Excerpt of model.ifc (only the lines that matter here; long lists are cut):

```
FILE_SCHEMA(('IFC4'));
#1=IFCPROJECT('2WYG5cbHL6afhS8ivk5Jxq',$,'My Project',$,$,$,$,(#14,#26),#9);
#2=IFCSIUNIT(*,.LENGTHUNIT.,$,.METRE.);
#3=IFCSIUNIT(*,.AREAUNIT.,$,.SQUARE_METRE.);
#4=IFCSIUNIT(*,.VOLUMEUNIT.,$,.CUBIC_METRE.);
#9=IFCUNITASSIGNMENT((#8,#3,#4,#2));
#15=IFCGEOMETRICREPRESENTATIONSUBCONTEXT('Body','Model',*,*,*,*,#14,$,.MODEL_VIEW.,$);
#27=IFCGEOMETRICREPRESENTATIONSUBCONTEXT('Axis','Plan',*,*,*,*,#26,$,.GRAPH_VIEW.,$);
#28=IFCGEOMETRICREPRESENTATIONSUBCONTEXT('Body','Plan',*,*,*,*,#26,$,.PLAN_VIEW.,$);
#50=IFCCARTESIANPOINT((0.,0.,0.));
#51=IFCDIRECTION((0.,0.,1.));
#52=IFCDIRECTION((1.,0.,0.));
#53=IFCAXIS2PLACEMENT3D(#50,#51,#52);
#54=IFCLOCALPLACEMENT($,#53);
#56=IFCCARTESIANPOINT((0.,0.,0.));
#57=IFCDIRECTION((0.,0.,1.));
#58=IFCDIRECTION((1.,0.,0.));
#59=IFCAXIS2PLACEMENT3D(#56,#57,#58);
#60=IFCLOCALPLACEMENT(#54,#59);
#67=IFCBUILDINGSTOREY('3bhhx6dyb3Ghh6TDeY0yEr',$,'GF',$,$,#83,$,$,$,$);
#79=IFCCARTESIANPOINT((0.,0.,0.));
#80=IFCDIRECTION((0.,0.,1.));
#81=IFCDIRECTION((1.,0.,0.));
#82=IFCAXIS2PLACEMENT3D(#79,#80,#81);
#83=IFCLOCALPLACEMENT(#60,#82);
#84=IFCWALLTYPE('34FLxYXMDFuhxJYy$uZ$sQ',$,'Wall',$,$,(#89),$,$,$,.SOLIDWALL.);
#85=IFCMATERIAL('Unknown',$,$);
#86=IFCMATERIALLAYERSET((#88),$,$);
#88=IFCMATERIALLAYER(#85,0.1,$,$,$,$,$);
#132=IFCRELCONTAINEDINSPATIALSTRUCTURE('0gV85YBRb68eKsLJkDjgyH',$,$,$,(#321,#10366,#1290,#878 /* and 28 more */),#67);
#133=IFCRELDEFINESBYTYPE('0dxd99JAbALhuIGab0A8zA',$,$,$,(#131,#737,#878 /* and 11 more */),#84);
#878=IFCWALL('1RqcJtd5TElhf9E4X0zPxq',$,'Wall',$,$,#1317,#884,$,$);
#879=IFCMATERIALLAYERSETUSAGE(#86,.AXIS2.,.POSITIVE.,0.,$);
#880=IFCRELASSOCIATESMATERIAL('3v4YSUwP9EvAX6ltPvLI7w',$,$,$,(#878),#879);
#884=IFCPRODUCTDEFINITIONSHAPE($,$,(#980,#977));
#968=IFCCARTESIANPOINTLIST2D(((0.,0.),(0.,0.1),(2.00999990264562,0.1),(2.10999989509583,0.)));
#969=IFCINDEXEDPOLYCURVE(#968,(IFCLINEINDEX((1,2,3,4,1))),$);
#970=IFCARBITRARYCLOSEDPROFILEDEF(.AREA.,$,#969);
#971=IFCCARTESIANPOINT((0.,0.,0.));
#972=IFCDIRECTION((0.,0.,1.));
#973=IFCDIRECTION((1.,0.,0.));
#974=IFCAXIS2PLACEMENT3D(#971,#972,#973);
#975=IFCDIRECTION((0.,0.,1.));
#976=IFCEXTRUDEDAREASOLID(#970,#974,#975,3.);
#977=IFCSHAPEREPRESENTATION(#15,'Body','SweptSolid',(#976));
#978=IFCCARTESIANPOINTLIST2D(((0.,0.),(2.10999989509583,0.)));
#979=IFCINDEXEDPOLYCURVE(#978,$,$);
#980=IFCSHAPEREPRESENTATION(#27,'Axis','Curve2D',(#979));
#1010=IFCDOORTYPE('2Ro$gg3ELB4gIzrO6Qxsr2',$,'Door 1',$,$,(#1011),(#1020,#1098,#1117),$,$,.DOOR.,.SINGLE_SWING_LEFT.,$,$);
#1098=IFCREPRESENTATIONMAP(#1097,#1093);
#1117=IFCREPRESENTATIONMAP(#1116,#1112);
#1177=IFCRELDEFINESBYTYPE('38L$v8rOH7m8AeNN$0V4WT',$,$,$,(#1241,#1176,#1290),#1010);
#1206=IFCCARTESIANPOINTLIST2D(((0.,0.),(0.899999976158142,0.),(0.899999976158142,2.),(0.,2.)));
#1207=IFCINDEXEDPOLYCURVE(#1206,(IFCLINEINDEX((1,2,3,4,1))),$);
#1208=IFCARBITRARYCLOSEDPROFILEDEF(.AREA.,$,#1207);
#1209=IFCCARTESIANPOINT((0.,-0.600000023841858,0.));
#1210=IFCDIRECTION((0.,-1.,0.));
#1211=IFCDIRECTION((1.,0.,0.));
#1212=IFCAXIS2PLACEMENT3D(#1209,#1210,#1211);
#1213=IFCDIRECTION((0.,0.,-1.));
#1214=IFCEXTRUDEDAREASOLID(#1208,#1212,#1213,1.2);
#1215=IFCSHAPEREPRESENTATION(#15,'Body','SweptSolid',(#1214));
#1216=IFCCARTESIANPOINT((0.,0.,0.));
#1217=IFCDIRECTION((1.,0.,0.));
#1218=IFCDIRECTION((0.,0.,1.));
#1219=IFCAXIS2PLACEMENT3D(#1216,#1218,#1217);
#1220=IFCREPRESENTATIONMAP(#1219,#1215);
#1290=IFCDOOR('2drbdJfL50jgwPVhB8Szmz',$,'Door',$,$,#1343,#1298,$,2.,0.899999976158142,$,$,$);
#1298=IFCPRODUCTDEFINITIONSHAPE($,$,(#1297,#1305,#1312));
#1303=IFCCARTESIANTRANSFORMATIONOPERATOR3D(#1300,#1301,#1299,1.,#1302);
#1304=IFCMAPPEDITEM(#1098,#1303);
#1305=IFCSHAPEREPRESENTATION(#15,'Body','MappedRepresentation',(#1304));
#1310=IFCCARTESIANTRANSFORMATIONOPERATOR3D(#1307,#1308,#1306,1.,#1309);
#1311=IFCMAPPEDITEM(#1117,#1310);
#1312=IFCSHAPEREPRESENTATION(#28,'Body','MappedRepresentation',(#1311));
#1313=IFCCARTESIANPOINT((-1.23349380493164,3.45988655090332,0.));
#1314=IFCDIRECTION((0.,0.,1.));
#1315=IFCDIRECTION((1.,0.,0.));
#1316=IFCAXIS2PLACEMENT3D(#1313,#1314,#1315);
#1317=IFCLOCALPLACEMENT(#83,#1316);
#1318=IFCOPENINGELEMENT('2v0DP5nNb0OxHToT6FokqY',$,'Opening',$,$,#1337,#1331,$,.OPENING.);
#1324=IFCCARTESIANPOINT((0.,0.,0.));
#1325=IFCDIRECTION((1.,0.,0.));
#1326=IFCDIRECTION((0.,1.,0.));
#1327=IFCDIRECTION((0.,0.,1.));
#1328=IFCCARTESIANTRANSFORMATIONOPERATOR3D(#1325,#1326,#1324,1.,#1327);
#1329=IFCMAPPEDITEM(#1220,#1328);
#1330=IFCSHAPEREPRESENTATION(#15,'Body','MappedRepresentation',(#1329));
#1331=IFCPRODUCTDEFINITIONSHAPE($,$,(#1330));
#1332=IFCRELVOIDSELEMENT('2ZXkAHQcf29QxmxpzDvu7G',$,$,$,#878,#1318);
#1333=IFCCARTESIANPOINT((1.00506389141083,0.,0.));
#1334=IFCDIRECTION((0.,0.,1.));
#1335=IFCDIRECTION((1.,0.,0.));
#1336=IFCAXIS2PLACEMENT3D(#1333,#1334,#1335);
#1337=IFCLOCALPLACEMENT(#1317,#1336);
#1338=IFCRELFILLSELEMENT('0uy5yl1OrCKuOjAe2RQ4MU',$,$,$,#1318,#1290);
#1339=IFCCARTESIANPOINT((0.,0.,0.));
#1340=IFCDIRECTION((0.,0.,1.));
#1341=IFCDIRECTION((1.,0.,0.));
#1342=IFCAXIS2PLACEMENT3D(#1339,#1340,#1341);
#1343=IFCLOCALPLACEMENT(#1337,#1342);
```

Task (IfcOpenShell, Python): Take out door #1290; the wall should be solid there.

```python
import ifcopenshell
import ifcopenshell.api.feature
import ifcopenshell.api.root
import ifcopenshell.geom
import ifcopenshell.util.shape

model = ifcopenshell.open("model.ifc")
settings = ifcopenshell.geom.settings()


def volume(element):
    """Net volume in cubic metres, openings subtracted."""
    shape = ifcopenshell.geom.create_shape(settings, element)
    return ifcopenshell.util.shape.get_volume(shape.geometry)


door = model.by_guid("2drbdJfL50jgwPVhB8Szmz")
opening = door.FillsVoids[0].RelatingOpeningElement
wall = opening.VoidsElements[0].RelatingBuildingElement
before = volume(wall)

ifcopenshell.api.root.remove_product(model, product=door)
ifcopenshell.api.feature.remove_feature(model, feature=opening)

after = volume(wall)

print(f"wall volume {before:.3f} -> {after:.3f} m3")

model.write("model_v2.ifc")
```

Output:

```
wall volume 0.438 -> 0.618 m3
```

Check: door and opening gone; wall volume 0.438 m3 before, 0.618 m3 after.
